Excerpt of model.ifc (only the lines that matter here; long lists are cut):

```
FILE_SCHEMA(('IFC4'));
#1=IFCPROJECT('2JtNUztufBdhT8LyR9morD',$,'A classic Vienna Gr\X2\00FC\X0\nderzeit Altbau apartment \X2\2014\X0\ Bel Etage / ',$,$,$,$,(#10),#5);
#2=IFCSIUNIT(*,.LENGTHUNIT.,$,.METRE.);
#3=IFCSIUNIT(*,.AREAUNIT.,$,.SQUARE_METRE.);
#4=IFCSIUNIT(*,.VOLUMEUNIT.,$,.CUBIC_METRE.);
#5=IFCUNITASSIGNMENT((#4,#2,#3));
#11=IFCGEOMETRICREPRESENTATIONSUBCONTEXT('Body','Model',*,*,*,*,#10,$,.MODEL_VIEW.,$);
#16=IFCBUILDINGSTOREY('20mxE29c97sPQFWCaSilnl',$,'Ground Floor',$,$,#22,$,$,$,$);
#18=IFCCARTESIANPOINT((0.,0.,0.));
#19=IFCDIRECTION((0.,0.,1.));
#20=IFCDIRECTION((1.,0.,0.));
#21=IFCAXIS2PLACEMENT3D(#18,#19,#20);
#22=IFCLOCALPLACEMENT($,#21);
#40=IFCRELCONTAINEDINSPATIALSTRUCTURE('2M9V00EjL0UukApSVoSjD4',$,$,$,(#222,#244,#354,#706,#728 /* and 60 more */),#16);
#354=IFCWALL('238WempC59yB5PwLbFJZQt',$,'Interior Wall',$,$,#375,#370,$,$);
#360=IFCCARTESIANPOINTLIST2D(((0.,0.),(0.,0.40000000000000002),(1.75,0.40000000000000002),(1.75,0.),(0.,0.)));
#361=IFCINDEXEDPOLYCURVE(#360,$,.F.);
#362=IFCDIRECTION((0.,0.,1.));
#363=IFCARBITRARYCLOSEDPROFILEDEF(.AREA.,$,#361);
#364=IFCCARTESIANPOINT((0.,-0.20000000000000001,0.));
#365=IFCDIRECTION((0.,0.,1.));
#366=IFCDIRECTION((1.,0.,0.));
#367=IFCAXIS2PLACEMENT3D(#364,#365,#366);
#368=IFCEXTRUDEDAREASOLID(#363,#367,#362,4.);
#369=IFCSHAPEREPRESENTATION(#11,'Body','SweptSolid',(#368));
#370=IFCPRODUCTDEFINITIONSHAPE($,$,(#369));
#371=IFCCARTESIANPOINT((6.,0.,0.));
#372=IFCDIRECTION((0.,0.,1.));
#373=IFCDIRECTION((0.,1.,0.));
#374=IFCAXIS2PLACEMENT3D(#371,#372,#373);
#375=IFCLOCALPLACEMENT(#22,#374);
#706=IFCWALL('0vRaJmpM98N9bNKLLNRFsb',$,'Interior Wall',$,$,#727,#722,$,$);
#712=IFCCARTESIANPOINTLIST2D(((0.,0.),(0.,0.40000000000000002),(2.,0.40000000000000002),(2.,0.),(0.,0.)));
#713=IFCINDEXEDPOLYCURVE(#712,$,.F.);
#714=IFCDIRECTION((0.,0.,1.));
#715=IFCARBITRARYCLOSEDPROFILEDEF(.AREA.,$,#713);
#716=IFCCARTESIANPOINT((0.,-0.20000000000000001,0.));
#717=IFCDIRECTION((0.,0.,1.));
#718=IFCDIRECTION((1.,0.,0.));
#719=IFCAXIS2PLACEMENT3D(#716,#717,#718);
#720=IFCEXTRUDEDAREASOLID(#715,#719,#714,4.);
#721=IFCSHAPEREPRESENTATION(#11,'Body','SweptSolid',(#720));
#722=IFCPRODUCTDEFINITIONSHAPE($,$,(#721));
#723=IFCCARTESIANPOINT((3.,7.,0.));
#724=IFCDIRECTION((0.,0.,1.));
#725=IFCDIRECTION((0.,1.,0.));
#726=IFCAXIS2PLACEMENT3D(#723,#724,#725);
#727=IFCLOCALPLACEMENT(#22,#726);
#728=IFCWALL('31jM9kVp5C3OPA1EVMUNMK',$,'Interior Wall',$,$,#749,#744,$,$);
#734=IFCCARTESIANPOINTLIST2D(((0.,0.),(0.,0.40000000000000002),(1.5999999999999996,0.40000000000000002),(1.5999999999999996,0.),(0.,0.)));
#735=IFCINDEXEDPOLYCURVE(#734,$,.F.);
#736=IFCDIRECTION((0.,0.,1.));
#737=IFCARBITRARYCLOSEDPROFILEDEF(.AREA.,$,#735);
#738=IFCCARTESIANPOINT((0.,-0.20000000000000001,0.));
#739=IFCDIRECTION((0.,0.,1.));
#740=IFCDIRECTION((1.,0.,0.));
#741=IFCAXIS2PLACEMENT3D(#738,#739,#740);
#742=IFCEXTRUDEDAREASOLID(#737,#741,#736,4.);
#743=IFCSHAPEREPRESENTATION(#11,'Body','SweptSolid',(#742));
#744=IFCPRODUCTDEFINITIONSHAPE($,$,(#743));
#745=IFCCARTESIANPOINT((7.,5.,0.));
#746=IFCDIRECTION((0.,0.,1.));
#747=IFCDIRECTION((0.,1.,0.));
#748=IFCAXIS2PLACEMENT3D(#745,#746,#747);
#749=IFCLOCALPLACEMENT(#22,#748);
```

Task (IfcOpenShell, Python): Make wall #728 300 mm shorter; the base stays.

```python
import ifcopenshell
import ifcopenshell.geom
import ifcopenshell.util.representation
import ifcopenshell.util.shape
import ifcopenshell.util.unit

model = ifcopenshell.open("model.ifc")
unit_scale = ifcopenshell.util.unit.calculate_unit_scale(model)
settings = ifcopenshell.geom.settings()


def volume(element):
    """Net volume in cubic metres, openings subtracted."""
    shape = ifcopenshell.geom.create_shape(settings, element)
    return ifcopenshell.util.shape.get_volume(shape.geometry)


wall = model.by_id(728)
before = volume(wall)

body = ifcopenshell.util.representation.get_representation(wall, "Model", "Body")
solid = body.Items[0]
old_height = solid.Depth
solid.Depth -= 0.3 / unit_scale
after = volume(wall)

print(f"height {old_height:g} -> {solid.Depth:g}, volume {before:.3f} -> {after:.3f} m3")

model.write("model_v2.ifc")
```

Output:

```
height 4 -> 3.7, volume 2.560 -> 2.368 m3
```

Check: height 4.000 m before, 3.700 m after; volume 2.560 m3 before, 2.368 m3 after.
